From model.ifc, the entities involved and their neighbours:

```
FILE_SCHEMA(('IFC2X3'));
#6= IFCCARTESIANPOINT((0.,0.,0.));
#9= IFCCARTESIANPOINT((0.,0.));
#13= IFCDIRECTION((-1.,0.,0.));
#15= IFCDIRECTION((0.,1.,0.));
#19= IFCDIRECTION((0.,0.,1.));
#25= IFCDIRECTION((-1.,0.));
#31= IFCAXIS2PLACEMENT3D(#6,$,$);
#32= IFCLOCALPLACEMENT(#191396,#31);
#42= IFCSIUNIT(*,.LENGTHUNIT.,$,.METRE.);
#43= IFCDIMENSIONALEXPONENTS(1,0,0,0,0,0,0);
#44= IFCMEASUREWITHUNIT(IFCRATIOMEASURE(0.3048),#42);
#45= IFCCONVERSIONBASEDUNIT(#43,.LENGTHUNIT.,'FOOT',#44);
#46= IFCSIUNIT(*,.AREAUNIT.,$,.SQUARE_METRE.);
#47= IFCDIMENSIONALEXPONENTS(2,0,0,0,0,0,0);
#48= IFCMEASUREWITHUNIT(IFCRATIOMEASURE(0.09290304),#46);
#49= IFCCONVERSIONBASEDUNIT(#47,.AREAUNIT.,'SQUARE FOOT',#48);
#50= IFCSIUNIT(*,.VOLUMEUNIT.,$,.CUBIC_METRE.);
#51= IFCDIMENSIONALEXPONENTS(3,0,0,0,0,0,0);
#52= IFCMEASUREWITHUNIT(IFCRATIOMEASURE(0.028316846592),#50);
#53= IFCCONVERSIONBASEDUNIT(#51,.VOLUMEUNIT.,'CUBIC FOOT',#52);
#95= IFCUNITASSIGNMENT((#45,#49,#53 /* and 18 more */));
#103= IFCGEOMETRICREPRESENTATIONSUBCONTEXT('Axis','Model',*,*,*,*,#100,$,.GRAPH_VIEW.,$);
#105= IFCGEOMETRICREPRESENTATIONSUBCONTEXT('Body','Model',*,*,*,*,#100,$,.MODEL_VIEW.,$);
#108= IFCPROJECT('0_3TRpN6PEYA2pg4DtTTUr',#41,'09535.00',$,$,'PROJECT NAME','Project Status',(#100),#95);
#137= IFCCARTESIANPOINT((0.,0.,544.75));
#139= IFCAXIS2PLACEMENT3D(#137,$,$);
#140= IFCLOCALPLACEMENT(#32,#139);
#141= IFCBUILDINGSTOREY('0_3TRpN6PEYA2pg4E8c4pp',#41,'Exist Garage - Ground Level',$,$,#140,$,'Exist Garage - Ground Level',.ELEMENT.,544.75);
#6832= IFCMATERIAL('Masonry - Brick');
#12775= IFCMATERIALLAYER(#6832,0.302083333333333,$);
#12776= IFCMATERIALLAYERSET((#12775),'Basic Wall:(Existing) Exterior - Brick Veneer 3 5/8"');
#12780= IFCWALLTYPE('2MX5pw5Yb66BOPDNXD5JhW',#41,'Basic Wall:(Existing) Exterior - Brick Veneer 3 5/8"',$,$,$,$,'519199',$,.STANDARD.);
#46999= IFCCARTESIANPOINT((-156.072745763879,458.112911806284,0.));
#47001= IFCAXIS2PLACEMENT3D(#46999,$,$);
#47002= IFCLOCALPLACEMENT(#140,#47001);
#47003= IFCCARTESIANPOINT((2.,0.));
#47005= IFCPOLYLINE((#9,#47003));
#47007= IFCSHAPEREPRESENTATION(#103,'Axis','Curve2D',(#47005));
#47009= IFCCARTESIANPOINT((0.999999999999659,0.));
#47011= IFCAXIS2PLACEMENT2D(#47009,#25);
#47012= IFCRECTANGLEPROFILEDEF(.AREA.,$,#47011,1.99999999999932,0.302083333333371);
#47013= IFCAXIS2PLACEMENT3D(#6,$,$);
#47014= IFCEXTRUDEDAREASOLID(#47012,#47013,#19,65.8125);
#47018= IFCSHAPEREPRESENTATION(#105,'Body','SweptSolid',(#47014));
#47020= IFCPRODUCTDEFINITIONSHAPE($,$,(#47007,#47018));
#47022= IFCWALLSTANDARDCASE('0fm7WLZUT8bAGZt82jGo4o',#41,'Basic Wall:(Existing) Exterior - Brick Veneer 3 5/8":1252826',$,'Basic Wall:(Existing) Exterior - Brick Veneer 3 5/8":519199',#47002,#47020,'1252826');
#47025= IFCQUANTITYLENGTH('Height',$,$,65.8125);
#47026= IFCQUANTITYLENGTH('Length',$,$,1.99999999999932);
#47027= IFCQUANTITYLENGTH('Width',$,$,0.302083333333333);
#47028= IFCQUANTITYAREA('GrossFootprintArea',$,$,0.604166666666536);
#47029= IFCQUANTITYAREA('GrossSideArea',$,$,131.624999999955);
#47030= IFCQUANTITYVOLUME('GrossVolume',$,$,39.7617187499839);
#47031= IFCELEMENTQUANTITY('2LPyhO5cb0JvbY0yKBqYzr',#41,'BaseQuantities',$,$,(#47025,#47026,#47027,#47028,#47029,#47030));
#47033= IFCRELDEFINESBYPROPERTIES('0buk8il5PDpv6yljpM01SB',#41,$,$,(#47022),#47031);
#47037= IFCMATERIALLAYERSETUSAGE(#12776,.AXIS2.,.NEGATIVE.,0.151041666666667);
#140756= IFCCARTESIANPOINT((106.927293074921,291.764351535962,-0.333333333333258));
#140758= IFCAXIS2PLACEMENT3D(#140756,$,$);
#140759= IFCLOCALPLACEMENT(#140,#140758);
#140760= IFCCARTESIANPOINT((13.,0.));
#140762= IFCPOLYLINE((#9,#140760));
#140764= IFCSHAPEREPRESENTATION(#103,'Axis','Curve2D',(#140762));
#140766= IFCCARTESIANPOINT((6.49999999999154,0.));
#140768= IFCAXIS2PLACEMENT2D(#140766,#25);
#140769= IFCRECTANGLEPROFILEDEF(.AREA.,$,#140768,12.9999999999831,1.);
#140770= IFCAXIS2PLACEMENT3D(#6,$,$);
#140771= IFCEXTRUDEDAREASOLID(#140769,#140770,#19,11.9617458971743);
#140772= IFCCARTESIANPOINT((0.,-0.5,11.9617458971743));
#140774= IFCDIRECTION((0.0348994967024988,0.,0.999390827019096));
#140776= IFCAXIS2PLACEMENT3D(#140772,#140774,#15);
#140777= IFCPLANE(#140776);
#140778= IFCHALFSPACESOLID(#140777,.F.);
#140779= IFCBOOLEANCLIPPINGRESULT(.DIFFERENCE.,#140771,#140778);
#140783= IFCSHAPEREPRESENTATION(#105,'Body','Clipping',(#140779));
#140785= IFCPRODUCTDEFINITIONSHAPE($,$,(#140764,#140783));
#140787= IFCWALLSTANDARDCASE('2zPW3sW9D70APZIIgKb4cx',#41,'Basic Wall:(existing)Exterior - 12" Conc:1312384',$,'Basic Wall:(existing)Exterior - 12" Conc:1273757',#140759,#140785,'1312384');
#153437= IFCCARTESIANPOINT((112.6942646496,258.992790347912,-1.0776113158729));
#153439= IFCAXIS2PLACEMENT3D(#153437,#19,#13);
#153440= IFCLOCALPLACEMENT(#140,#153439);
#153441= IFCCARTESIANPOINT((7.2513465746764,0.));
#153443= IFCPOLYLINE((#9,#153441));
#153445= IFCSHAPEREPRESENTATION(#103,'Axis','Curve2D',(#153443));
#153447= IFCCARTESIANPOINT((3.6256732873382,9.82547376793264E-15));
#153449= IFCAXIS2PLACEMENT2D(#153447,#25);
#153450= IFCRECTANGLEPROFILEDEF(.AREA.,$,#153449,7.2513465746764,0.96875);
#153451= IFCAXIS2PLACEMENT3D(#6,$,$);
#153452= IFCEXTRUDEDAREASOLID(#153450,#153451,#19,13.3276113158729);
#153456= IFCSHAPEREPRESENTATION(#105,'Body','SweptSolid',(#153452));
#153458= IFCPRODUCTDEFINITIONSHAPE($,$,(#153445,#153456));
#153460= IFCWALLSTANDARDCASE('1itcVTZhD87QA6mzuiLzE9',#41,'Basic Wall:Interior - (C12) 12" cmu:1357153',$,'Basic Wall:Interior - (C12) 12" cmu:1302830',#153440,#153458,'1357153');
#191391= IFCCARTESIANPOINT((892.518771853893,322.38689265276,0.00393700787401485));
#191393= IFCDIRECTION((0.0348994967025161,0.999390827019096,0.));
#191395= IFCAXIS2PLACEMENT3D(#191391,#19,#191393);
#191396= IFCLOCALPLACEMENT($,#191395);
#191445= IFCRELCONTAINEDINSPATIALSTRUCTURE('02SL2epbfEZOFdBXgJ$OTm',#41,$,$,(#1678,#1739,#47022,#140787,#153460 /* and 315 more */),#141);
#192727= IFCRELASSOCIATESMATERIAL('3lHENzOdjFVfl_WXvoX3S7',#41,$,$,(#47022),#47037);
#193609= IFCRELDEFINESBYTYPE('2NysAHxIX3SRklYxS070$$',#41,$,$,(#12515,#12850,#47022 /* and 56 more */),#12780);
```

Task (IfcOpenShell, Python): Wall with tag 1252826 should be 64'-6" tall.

```python
import ifcopenshell
import ifcopenshell.api.pset
import ifcopenshell.geom
import ifcopenshell.util.element
import ifcopenshell.util.representation
import ifcopenshell.util.shape
import ifcopenshell.util.unit

model = ifcopenshell.open("model.ifc")
unit_scale = ifcopenshell.util.unit.calculate_unit_scale(model)
area_scale = ifcopenshell.util.unit.calculate_unit_scale(model, "AREAUNIT")
volume_scale = ifcopenshell.util.unit.calculate_unit_scale(model, "VOLUMEUNIT")
settings = ifcopenshell.geom.settings()


def volume(element):
    """Net volume in cubic metres, openings subtracted."""
    shape = ifcopenshell.geom.create_shape(settings, element)
    return ifcopenshell.util.shape.get_volume(shape.geometry)


wall = model.by_id(47022)
before = volume(wall)

body = ifcopenshell.util.representation.get_representation(wall, "Model", "Body")
solid = body.Items[0]
old_height = solid.Depth
solid.Depth = 774 * 0.0254 / unit_scale
after = volume(wall)

# Update the stored height, areas and volumes.
qto = model.by_id(ifcopenshell.util.element.get_pset(wall, "BaseQuantities", should_inherit=False)["id"])
ifcopenshell.api.pset.edit_qto(model, qto=qto, properties={
    "Height": solid.Depth,
    "GrossSideArea": ifcopenshell.util.element.get_pset(wall, "BaseQuantities", "GrossSideArea") * solid.Depth / old_height,
    "GrossVolume": ifcopenshell.util.element.get_pset(wall, "BaseQuantities", "GrossVolume") * solid.Depth / old_height,
})

print(f"height {old_height:g} -> {solid.Depth:g}, volume {before:.3f} -> {after:.3f} m3")

model.write("model_rev.ifc")
```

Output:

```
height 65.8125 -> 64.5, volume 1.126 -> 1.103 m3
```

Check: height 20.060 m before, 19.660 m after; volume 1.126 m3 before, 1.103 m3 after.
